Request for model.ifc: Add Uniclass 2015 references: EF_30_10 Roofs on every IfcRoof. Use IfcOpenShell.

First a look at what the model holds.

```python
import ifcopenshell

model = ifcopenshell.open("model.ifc")
print(model.schema)
print("classifications:", [c.Name for c in model.by_type("IfcClassification")])
for ifc_class in ("IfcDoor", "IfcRoof", "IfcStair", "IfcWall", "IfcWindow"):
    print(ifc_class, len(model.by_type(ifc_class)))
```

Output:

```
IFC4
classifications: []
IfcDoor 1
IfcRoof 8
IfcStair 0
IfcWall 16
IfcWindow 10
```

```python
import ifcopenshell
import ifcopenshell.api.classification

model = ifcopenshell.open("model.ifc")

system = ifcopenshell.api.classification.add_classification(model, classification="Uniclass 2015")

codes = {
    "IfcRoof": ("EF_30_10", "Roofs"),
}
for ifc_class, (code, name) in codes.items():
    products = model.by_type(ifc_class)
    ifcopenshell.api.classification.add_reference(
        model, products=products, classification=system, identification=code, name=name
    )
    print(code, len(products))

model.write("model-out.ifc")
```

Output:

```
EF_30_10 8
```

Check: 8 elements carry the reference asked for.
